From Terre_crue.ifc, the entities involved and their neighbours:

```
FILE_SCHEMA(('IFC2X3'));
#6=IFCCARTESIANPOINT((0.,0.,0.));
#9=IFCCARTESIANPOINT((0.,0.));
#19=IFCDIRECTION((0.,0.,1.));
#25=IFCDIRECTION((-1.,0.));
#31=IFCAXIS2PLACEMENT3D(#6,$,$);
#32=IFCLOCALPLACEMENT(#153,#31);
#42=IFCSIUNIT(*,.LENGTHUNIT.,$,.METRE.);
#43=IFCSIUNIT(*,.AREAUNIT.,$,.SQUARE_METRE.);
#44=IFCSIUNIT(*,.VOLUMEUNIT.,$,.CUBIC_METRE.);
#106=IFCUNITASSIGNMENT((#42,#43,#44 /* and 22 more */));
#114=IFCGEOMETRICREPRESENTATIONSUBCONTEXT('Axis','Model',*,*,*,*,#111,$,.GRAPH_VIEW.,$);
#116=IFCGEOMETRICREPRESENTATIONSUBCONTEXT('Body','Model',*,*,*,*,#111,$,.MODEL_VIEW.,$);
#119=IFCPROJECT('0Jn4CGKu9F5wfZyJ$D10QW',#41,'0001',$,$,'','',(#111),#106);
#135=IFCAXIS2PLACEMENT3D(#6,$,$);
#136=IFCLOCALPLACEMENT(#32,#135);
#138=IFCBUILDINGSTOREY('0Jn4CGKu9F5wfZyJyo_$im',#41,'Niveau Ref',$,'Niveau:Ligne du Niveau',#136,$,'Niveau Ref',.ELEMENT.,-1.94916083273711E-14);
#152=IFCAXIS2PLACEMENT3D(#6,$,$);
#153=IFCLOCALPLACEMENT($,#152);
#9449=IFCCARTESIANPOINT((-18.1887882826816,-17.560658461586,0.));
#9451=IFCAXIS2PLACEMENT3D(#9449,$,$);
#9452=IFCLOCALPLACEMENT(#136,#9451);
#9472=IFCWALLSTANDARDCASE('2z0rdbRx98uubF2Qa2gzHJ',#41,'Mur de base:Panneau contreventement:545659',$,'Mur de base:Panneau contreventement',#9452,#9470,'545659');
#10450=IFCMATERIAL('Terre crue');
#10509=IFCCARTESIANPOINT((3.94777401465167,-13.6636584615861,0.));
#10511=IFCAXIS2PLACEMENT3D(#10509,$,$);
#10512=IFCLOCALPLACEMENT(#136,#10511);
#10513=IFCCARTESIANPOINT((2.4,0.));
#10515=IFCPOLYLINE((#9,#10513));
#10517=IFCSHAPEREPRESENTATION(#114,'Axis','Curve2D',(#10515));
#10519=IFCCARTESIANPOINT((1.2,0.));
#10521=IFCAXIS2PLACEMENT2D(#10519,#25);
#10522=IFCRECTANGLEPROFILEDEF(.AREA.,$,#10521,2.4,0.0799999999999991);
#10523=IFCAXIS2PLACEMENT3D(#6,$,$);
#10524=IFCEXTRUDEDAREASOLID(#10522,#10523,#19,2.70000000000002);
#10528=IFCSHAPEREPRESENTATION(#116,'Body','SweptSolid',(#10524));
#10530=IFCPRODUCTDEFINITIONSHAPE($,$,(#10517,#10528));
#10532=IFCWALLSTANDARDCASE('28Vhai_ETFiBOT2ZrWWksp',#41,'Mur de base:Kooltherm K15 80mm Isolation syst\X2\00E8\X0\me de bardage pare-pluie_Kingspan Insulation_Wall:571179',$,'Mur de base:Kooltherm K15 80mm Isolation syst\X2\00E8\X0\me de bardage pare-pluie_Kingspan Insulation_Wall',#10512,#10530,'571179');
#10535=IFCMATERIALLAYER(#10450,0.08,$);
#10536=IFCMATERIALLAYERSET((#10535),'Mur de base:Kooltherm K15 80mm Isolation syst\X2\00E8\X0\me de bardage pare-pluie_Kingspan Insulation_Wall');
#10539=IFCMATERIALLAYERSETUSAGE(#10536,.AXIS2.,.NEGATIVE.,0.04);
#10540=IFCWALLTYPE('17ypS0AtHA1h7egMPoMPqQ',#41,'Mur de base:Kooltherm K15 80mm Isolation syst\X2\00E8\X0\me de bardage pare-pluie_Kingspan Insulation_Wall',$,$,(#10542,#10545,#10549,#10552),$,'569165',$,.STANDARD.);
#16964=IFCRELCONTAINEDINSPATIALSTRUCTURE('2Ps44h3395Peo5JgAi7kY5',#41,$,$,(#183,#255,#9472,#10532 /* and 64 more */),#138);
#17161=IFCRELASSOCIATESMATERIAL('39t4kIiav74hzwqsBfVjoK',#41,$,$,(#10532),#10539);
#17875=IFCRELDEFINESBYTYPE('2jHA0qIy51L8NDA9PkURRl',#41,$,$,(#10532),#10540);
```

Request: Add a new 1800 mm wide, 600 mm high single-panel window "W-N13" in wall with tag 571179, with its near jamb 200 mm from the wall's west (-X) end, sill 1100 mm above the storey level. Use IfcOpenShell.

```python
import numpy as np
import ifcopenshell
import ifcopenshell.api.feature
import ifcopenshell.api.geometry
import ifcopenshell.api.root
import ifcopenshell.api.spatial
import ifcopenshell.api.type
import ifcopenshell.geom
import ifcopenshell.util.element
import ifcopenshell.util.placement
import ifcopenshell.util.representation
import ifcopenshell.util.shape
import ifcopenshell.util.unit

model = ifcopenshell.open("Terre_crue.ifc")
unit_scale = ifcopenshell.util.unit.calculate_unit_scale(model)
settings = ifcopenshell.geom.settings()


def volume(element):
    """Net volume in cubic metres, openings subtracted."""
    shape = ifcopenshell.geom.create_shape(settings, element)
    return ifcopenshell.util.shape.get_volume(shape.geometry)


wall = model.by_guid("28Vhai_ETFiBOT2ZrWWksp")
storey = ifcopenshell.util.element.get_container(wall, ifc_class="IfcBuildingStorey")
context = ifcopenshell.util.representation.get_context(model, "Model", "Body", "MODEL_VIEW")
before = volume(wall)

width, height, from_end, sill = 1.8, 0.6, 0.2, 1.1  # metres

# The wall runs along its own X axis, and the end named is its -X end.
wall_shape = ifcopenshell.geom.create_shape(settings, wall)
x, y, z = ifcopenshell.util.shape.get_vertices(wall_shape.geometry).T
start = x.min() + from_end
face, thickness = float(y.min()), float(y.max() - y.min())
wall_matrix = ifcopenshell.util.placement.get_local_placement(wall.ObjectPlacement)
level = ifcopenshell.util.placement.get_local_placement(storey.ObjectPlacement)[2, 3]


def in_wall(x, y):
    """Placement at x, y metres in the wall's axes, at sill height."""
    matrix = wall_matrix.copy()
    matrix[:, 3] = wall_matrix @ np.array([x / unit_scale, y / unit_scale, 0.0, 1.0])
    matrix[2, 3] = level + sill / unit_scale
    return matrix


# Opening: a box that overshoots both wall faces by 50 mm.
opening = ifcopenshell.api.root.create_entity(model, ifc_class="IfcOpeningElement")
box = ifcopenshell.api.geometry.add_wall_representation(
    model, context=context, length=width, height=height, thickness=thickness + 0.1
)
ifcopenshell.api.geometry.assign_representation(model, product=opening, representation=box)
ifcopenshell.api.geometry.edit_object_placement(model, product=opening, matrix=in_wall(start, face - 0.05), is_si=False)
ifcopenshell.api.feature.add_feature(model, feature=opening, element=wall)

window = ifcopenshell.api.root.create_entity(model, ifc_class="IfcWindow", name="W-N13")
window.OverallWidth, window.OverallHeight = width / unit_scale, height / unit_scale
body = ifcopenshell.api.geometry.add_window_representation(
    model,
    context=context,
    overall_width=window.OverallWidth,
    overall_height=window.OverallHeight,
    partition_type="SINGLE_PANEL",
)
ifcopenshell.api.geometry.assign_representation(model, product=window, representation=body)
ifcopenshell.api.spatial.assign_container(model, products=[window], relating_structure=storey)
fills = ifcopenshell.api.feature.add_filling(model, opening=opening, element=window)
fills.OwnerHistory = window.OwnerHistory  # required in IFC2X3

# IFC2X3 keeps the operation on the window style.
style = ifcopenshell.api.root.create_entity(model, ifc_class="IfcWindowStyle", name="W-N13")
style.OperationType, style.ConstructionType = "SINGLE_PANEL", "NOTDEFINED"
style.ParameterTakesPrecedence = style.Sizeable = False
ifcopenshell.api.type.assign_type(model, related_objects=[window], relating_type=style)

# Centre the window in the wall's thickness.
ifcopenshell.api.geometry.edit_object_placement(model, product=window, matrix=in_wall(start, face), is_si=False)
window_shape = ifcopenshell.geom.create_shape(settings, window)
depth = ifcopenshell.util.shape.get_vertices(window_shape.geometry)[:, 1]
offset = face + thickness / 2 - (depth.min() + depth.max()) / 2
ifcopenshell.api.geometry.edit_object_placement(model, product=window, matrix=in_wall(start, offset), is_si=False)

after = volume(wall)

print(f"wall volume {before:.3f} -> {after:.3f} m3")

model.write("Terre_crue_v2.ifc")
```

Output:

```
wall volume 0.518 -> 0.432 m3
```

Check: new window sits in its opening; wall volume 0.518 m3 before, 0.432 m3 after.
